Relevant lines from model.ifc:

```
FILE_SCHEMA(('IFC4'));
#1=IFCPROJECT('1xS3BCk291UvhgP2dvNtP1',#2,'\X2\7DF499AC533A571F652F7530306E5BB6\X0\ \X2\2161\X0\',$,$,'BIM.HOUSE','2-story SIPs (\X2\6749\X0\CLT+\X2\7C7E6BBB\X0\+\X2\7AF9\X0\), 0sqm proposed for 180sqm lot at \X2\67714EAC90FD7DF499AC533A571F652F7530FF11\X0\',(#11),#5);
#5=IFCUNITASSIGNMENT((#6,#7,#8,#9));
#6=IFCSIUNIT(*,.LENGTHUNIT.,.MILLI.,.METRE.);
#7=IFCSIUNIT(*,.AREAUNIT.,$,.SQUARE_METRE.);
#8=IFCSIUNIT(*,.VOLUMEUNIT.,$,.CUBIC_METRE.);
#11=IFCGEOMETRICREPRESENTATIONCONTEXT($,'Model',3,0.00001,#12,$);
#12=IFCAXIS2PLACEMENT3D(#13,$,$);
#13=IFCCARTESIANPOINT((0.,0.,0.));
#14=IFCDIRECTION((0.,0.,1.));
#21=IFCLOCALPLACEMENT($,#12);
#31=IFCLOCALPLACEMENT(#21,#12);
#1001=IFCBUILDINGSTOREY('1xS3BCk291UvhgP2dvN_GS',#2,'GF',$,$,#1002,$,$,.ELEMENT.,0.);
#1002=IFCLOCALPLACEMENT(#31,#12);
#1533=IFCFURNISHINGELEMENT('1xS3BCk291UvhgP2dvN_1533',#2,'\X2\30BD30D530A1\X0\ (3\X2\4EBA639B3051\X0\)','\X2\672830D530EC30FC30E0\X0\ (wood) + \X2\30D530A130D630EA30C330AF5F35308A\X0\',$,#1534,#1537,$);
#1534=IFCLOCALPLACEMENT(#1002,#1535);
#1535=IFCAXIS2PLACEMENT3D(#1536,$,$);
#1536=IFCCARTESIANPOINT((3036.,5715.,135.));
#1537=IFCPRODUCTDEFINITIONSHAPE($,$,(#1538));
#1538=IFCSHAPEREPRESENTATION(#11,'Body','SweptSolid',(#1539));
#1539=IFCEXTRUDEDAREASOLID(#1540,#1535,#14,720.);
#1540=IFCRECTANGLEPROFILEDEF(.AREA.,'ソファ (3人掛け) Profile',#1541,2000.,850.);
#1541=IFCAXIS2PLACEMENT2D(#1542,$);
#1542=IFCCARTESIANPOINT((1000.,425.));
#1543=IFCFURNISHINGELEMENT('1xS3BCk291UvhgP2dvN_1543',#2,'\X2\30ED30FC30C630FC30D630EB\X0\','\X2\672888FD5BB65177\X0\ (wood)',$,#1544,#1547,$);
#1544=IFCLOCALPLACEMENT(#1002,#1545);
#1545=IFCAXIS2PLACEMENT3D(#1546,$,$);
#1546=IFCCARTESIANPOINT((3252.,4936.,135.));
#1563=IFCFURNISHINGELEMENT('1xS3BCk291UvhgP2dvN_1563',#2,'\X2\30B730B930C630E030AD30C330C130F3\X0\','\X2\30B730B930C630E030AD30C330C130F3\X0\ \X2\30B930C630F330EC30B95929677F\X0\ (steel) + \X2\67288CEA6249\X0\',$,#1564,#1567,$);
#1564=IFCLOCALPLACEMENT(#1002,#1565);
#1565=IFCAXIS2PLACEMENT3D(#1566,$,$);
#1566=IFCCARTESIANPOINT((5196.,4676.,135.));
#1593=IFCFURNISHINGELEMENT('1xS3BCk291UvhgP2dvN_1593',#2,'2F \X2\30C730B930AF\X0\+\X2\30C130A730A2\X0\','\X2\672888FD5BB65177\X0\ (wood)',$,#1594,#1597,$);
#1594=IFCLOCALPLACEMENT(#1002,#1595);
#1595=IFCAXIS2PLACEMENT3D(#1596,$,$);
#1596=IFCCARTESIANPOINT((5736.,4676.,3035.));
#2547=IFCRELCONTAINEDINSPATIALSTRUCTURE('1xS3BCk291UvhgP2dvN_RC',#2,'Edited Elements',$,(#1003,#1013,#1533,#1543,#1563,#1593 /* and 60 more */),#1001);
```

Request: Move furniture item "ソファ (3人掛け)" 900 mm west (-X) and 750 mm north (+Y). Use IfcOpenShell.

```python
import ifcopenshell
import ifcopenshell.api.geometry
import ifcopenshell.util.placement

model = ifcopenshell.open("model.ifc")

item = model.by_guid("1xS3BCk291UvhgP2dvN_1533")
matrix = ifcopenshell.util.placement.get_local_placement(item.ObjectPlacement)
matrix[0, 3] -= 900.0
matrix[1, 3] += 750.0
ifcopenshell.api.geometry.edit_object_placement(model, product=item, matrix=matrix, is_si=False)

print(ifcopenshell.util.placement.get_local_placement(item.ObjectPlacement).round(3) + 0.0)

model.write("model-out.ifc")
```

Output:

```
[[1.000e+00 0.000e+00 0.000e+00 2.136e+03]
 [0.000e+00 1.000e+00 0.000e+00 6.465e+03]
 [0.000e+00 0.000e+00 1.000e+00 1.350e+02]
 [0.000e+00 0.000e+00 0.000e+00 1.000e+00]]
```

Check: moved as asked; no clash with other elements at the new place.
